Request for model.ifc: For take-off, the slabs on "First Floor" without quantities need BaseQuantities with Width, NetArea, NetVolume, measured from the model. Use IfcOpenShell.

First a look at what the model holds.

```python
import ifcopenshell
import ifcopenshell.util.element
import ifcopenshell.util.unit

model = ifcopenshell.open("model.ifc")
print(model.schema)
for unit_type in ("LENGTHUNIT", "AREAUNIT", "VOLUMEUNIT"):
    print(unit_type, ifcopenshell.util.unit.calculate_unit_scale(model, unit_type))
storey = next(s for s in model.by_type("IfcBuildingStorey") if s.Name == "First Floor")
slabs = [e for e in ifcopenshell.util.element.get_decomposition(storey) if e.is_a("IfcSlab")]
for e in sorted(slabs, key=lambda e: e.id()):
    print(e.id(), e.is_a(), e.Name, list(ifcopenshell.util.element.get_psets(e, qtos_only=True)), sep=" | ")
```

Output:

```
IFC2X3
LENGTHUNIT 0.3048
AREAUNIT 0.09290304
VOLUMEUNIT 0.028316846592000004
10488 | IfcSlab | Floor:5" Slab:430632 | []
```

```python
import ifcopenshell
import ifcopenshell.api.pset
import ifcopenshell.geom
import ifcopenshell.util.element
import ifcopenshell.util.shape
import ifcopenshell.util.unit

model = ifcopenshell.open("model.ifc")
unit_scale = ifcopenshell.util.unit.calculate_unit_scale(model)
area_scale = ifcopenshell.util.unit.calculate_unit_scale(model, "AREAUNIT")
volume_scale = ifcopenshell.util.unit.calculate_unit_scale(model, "VOLUMEUNIT")
settings = ifcopenshell.geom.settings()

storey = next(s for s in model.by_type("IfcBuildingStorey") if s.Name == "First Floor")
slabs = [e for e in ifcopenshell.util.element.get_decomposition(storey) if e.is_a("IfcSlab")]

for e in sorted(slabs, key=lambda e: e.id()):
    if ifcopenshell.util.element.get_psets(e, qtos_only=True, should_inherit=False):
        continue
    # Geometry comes back in metres, in the element's own axes.
    shape = ifcopenshell.geom.create_shape(settings, e)
    values = {
        "Width": ifcopenshell.util.shape.get_z(shape.geometry) / unit_scale,
        "NetArea": ifcopenshell.util.shape.get_footprint_area(shape.geometry) / area_scale,
        "NetVolume": ifcopenshell.util.shape.get_volume(shape.geometry) / volume_scale,
    }
    qto = ifcopenshell.api.pset.add_qto(model, product=e, name="BaseQuantities")
    ifcopenshell.api.pset.edit_qto(model, qto=qto, properties=values)
    print(e.id(), {k: round(v, 3) for k, v in values.items()})

model.write("model_edited.ifc")
```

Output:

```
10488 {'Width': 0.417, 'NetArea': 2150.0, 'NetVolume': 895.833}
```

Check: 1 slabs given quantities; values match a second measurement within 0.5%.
